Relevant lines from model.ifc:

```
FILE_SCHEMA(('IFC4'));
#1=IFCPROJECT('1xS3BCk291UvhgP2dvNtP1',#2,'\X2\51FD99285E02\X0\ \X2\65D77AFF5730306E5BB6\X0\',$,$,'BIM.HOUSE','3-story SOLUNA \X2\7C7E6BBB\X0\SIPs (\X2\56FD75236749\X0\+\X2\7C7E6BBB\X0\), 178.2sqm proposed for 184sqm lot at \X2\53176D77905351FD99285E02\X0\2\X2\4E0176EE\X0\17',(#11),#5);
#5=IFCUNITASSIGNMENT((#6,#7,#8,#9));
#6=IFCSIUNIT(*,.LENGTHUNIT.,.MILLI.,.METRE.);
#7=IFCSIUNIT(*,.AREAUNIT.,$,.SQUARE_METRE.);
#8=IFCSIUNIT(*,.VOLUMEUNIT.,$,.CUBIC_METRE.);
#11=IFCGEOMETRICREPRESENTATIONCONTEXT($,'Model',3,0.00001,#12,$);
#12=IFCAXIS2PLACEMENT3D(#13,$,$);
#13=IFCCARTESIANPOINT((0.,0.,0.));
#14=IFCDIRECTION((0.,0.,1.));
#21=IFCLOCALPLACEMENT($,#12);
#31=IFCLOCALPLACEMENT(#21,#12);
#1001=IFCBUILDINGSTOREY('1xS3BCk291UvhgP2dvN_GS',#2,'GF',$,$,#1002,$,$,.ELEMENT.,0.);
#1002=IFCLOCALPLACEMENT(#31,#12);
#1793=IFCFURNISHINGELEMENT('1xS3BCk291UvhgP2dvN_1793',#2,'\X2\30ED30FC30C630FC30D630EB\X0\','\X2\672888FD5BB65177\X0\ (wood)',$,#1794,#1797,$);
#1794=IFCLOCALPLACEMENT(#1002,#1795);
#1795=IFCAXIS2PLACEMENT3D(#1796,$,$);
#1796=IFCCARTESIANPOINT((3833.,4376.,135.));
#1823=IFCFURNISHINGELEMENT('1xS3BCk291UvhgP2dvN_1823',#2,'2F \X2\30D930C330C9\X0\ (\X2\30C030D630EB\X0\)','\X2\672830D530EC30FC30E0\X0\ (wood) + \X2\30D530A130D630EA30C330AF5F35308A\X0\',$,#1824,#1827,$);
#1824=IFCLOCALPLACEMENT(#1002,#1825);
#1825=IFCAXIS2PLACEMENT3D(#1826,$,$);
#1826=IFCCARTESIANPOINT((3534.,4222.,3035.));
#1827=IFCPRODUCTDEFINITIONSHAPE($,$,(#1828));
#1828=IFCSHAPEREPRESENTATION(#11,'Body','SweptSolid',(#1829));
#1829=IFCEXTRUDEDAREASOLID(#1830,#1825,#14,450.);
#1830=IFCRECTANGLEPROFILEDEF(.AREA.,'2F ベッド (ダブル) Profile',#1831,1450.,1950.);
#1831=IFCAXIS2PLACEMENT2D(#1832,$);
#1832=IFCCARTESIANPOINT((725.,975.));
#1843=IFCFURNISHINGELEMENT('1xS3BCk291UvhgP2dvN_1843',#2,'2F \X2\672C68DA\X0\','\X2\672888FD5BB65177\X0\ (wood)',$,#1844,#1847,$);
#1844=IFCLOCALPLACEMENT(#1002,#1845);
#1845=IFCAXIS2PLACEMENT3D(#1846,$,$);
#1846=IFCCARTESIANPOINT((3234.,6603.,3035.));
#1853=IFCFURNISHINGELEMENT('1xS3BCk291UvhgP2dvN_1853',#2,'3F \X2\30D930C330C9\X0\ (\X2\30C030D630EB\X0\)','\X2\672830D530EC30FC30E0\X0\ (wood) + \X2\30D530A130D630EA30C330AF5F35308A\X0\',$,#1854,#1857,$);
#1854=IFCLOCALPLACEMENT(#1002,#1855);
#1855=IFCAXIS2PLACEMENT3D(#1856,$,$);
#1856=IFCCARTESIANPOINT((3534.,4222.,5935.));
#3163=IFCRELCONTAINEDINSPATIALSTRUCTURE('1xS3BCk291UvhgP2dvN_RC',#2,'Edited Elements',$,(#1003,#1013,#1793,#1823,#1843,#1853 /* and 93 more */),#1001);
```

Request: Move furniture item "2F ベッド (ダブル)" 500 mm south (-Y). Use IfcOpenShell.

```python
import ifcopenshell
import ifcopenshell.api.geometry
import ifcopenshell.util.placement
import ifcopenshell.util.unit

model = ifcopenshell.open("model.ifc")
unit_scale = ifcopenshell.util.unit.calculate_unit_scale(model)

item = model.by_guid("1xS3BCk291UvhgP2dvN_1823")
matrix = ifcopenshell.util.placement.get_local_placement(item.ObjectPlacement)
matrix[1, 3] -= 0.5 / unit_scale
ifcopenshell.api.geometry.edit_object_placement(model, product=item, matrix=matrix, is_si=False)

print(ifcopenshell.util.placement.get_local_placement(item.ObjectPlacement).round(3) + 0.0)

model.write("model-out.ifc")
```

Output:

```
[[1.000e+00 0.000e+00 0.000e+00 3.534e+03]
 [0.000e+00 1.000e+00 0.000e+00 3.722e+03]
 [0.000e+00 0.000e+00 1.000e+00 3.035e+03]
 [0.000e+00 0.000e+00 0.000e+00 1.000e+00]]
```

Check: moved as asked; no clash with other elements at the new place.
